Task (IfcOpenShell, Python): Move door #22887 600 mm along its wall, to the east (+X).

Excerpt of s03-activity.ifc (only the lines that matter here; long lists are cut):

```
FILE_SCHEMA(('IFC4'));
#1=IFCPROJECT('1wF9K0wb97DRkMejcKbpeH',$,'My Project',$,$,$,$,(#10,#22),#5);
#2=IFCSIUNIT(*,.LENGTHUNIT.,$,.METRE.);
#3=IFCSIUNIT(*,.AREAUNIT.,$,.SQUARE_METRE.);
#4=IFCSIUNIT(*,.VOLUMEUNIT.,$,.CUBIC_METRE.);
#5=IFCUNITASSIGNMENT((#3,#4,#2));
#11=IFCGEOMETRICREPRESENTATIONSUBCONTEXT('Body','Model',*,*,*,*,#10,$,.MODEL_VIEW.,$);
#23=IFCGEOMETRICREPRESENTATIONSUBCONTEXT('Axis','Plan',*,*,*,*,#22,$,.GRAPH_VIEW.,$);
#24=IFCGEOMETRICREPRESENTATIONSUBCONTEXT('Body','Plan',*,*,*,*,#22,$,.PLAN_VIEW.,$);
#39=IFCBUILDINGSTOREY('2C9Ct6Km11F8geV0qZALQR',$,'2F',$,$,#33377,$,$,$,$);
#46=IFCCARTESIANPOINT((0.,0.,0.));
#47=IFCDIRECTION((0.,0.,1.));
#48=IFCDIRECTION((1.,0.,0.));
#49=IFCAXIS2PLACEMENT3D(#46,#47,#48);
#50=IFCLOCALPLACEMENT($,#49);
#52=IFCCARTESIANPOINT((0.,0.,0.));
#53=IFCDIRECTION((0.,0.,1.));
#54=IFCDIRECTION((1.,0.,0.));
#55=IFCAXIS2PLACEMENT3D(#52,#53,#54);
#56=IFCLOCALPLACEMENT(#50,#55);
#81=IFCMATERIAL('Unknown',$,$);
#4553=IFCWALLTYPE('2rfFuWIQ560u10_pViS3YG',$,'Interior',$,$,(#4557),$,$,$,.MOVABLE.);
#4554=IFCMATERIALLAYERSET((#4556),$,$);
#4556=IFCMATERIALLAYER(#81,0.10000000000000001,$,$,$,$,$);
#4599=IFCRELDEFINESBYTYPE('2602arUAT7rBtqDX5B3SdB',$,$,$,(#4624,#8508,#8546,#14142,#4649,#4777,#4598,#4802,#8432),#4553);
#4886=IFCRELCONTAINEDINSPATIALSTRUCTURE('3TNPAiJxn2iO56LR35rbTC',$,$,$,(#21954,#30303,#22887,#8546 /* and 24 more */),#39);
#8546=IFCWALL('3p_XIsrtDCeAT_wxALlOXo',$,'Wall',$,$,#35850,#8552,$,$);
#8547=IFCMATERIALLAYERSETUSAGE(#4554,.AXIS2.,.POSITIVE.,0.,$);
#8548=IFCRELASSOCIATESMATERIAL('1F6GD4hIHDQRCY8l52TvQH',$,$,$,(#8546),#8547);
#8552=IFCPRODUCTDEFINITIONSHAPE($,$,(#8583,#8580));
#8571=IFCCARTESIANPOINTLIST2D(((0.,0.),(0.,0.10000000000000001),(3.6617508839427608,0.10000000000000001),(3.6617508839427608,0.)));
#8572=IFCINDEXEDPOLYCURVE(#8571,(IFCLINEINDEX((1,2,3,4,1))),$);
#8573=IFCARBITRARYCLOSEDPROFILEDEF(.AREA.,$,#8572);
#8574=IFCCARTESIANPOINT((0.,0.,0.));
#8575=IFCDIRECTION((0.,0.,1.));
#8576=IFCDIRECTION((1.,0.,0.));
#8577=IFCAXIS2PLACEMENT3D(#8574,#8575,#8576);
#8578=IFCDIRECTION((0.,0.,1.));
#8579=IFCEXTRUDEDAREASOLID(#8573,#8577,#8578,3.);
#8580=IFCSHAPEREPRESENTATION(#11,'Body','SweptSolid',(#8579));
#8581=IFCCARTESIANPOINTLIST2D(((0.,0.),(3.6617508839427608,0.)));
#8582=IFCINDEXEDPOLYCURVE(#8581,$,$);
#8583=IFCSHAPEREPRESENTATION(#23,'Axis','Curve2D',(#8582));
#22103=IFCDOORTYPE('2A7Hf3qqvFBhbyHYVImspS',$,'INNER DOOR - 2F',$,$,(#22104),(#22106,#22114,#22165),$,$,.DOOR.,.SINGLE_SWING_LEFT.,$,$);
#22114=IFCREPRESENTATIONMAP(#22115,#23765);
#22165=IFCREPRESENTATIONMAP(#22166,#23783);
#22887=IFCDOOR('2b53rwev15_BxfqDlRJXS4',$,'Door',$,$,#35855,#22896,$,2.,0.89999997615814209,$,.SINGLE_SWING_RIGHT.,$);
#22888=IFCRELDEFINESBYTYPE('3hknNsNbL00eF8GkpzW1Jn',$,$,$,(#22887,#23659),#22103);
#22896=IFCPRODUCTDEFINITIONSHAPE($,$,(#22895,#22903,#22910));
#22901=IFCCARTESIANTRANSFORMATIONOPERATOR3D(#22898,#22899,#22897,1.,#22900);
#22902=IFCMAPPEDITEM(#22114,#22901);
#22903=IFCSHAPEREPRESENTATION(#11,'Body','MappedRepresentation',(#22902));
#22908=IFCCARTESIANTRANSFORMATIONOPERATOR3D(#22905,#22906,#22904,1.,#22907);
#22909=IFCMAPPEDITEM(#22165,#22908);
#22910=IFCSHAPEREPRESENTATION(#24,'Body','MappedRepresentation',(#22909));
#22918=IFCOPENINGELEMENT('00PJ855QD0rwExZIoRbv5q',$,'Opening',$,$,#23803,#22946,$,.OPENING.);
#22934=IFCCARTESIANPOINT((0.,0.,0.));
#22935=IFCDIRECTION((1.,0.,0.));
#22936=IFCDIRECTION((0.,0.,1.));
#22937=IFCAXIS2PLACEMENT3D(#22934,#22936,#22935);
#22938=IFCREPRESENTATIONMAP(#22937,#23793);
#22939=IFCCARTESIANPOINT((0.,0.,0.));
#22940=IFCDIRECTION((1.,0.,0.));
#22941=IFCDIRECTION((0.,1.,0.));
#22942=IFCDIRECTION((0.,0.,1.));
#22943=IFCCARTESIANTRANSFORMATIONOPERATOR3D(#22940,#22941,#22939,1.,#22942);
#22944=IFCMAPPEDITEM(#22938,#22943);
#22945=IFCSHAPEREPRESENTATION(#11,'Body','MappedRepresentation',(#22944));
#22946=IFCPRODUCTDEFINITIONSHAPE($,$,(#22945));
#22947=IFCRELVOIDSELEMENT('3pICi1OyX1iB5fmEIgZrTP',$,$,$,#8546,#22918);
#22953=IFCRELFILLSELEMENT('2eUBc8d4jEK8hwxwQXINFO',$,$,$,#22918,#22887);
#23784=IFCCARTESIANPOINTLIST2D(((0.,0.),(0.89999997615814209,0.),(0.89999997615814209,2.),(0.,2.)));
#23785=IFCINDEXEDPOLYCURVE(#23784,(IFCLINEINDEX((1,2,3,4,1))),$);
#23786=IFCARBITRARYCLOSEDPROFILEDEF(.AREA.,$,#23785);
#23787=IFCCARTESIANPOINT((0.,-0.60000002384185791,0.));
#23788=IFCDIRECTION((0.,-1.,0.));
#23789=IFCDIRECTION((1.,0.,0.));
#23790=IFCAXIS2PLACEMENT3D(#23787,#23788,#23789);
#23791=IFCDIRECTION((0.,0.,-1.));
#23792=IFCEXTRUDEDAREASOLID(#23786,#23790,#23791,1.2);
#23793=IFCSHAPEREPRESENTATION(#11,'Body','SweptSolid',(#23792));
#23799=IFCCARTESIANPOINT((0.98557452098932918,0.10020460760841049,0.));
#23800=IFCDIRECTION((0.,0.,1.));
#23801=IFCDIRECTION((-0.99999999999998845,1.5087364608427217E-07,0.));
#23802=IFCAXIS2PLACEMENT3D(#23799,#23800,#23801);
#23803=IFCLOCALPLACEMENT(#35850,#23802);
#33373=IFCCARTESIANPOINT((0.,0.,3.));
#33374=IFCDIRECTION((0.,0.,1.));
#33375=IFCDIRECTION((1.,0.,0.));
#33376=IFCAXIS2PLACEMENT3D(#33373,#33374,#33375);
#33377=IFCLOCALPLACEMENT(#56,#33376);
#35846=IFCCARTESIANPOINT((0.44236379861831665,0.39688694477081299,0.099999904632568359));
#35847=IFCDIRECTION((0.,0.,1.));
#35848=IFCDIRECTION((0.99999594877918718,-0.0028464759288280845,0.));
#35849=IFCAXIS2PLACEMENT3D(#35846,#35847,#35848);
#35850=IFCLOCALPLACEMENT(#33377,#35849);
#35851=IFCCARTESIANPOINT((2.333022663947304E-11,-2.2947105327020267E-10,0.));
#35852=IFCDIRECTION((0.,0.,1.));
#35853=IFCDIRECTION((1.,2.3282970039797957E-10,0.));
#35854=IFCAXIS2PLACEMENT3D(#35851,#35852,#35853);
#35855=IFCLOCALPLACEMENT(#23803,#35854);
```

```python
import ifcopenshell
import ifcopenshell.api.geometry
import ifcopenshell.util.placement
import ifcopenshell.util.unit

model = ifcopenshell.open("s03-activity.ifc")
unit_scale = ifcopenshell.util.unit.calculate_unit_scale(model)

door = model.by_guid("2b53rwev15_BxfqDlRJXS4")
opening = door.FillsVoids[0].RelatingOpeningElement
wall = opening.VoidsElements[0].RelatingBuildingElement

wall_matrix = ifcopenshell.util.placement.get_local_placement(wall.ObjectPlacement)
shift = wall_matrix[:3, 0] * 0.6 / unit_scale
before = ifcopenshell.util.placement.get_local_placement(door.ObjectPlacement)[:3, 3].copy()

# The door is placed relative to its opening, so it follows when the opening moves.
matrix = ifcopenshell.util.placement.get_local_placement(opening.ObjectPlacement)
matrix[:3, 3] += shift
ifcopenshell.api.geometry.edit_object_placement(
    model, product=opening, matrix=matrix, is_si=False, should_transform_children=True
)

after = ifcopenshell.util.placement.get_local_placement(door.ObjectPlacement)[:3, 3]
print("door moved by", (after - before).round(3) + 0.0)

model.write("s03-activity-out.ifc")
```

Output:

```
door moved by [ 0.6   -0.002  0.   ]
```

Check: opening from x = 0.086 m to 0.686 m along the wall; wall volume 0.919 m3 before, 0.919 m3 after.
